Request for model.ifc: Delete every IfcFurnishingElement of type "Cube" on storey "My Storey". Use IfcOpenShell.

First a look at what the model holds.

```python
import ifcopenshell
import ifcopenshell.util.element

model = ifcopenshell.open("model.ifc")
print(model.schema)
storey = next(s for s in model.by_type("IfcBuildingStorey") if s.Name == "My Storey")
furniture = [e for e in ifcopenshell.util.element.get_decomposition(storey) if e.is_a("IfcFurnishingElement")]
seen = {}
for e in furniture:
    element_type = ifcopenshell.util.element.get_type(e)
    name = element_type.Name if element_type not in (None, e) else None
    seen[name] = seen.get(name, 0) + 1
for name, count in sorted(seen.items(), key=str):
    print(count, "x", name)
```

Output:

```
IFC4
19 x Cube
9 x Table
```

```python
import ifcopenshell
import ifcopenshell.api.root
import ifcopenshell.util.element

model = ifcopenshell.open("model.ifc")

storey = next(s for s in model.by_type("IfcBuildingStorey") if s.Name == "My Storey")
furniture = [e for e in ifcopenshell.util.element.get_decomposition(storey) if e.is_a("IfcFurnishingElement")]
targets = [e for e in furniture if (t := ifcopenshell.util.element.get_type(e)) not in (None, e) and t.Name == "Cube"]

for e in targets:
    ifcopenshell.api.root.remove_product(model, product=e)
print(len(targets), "removed")

model.write("model_edited.ifc")
```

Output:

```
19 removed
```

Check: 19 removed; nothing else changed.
